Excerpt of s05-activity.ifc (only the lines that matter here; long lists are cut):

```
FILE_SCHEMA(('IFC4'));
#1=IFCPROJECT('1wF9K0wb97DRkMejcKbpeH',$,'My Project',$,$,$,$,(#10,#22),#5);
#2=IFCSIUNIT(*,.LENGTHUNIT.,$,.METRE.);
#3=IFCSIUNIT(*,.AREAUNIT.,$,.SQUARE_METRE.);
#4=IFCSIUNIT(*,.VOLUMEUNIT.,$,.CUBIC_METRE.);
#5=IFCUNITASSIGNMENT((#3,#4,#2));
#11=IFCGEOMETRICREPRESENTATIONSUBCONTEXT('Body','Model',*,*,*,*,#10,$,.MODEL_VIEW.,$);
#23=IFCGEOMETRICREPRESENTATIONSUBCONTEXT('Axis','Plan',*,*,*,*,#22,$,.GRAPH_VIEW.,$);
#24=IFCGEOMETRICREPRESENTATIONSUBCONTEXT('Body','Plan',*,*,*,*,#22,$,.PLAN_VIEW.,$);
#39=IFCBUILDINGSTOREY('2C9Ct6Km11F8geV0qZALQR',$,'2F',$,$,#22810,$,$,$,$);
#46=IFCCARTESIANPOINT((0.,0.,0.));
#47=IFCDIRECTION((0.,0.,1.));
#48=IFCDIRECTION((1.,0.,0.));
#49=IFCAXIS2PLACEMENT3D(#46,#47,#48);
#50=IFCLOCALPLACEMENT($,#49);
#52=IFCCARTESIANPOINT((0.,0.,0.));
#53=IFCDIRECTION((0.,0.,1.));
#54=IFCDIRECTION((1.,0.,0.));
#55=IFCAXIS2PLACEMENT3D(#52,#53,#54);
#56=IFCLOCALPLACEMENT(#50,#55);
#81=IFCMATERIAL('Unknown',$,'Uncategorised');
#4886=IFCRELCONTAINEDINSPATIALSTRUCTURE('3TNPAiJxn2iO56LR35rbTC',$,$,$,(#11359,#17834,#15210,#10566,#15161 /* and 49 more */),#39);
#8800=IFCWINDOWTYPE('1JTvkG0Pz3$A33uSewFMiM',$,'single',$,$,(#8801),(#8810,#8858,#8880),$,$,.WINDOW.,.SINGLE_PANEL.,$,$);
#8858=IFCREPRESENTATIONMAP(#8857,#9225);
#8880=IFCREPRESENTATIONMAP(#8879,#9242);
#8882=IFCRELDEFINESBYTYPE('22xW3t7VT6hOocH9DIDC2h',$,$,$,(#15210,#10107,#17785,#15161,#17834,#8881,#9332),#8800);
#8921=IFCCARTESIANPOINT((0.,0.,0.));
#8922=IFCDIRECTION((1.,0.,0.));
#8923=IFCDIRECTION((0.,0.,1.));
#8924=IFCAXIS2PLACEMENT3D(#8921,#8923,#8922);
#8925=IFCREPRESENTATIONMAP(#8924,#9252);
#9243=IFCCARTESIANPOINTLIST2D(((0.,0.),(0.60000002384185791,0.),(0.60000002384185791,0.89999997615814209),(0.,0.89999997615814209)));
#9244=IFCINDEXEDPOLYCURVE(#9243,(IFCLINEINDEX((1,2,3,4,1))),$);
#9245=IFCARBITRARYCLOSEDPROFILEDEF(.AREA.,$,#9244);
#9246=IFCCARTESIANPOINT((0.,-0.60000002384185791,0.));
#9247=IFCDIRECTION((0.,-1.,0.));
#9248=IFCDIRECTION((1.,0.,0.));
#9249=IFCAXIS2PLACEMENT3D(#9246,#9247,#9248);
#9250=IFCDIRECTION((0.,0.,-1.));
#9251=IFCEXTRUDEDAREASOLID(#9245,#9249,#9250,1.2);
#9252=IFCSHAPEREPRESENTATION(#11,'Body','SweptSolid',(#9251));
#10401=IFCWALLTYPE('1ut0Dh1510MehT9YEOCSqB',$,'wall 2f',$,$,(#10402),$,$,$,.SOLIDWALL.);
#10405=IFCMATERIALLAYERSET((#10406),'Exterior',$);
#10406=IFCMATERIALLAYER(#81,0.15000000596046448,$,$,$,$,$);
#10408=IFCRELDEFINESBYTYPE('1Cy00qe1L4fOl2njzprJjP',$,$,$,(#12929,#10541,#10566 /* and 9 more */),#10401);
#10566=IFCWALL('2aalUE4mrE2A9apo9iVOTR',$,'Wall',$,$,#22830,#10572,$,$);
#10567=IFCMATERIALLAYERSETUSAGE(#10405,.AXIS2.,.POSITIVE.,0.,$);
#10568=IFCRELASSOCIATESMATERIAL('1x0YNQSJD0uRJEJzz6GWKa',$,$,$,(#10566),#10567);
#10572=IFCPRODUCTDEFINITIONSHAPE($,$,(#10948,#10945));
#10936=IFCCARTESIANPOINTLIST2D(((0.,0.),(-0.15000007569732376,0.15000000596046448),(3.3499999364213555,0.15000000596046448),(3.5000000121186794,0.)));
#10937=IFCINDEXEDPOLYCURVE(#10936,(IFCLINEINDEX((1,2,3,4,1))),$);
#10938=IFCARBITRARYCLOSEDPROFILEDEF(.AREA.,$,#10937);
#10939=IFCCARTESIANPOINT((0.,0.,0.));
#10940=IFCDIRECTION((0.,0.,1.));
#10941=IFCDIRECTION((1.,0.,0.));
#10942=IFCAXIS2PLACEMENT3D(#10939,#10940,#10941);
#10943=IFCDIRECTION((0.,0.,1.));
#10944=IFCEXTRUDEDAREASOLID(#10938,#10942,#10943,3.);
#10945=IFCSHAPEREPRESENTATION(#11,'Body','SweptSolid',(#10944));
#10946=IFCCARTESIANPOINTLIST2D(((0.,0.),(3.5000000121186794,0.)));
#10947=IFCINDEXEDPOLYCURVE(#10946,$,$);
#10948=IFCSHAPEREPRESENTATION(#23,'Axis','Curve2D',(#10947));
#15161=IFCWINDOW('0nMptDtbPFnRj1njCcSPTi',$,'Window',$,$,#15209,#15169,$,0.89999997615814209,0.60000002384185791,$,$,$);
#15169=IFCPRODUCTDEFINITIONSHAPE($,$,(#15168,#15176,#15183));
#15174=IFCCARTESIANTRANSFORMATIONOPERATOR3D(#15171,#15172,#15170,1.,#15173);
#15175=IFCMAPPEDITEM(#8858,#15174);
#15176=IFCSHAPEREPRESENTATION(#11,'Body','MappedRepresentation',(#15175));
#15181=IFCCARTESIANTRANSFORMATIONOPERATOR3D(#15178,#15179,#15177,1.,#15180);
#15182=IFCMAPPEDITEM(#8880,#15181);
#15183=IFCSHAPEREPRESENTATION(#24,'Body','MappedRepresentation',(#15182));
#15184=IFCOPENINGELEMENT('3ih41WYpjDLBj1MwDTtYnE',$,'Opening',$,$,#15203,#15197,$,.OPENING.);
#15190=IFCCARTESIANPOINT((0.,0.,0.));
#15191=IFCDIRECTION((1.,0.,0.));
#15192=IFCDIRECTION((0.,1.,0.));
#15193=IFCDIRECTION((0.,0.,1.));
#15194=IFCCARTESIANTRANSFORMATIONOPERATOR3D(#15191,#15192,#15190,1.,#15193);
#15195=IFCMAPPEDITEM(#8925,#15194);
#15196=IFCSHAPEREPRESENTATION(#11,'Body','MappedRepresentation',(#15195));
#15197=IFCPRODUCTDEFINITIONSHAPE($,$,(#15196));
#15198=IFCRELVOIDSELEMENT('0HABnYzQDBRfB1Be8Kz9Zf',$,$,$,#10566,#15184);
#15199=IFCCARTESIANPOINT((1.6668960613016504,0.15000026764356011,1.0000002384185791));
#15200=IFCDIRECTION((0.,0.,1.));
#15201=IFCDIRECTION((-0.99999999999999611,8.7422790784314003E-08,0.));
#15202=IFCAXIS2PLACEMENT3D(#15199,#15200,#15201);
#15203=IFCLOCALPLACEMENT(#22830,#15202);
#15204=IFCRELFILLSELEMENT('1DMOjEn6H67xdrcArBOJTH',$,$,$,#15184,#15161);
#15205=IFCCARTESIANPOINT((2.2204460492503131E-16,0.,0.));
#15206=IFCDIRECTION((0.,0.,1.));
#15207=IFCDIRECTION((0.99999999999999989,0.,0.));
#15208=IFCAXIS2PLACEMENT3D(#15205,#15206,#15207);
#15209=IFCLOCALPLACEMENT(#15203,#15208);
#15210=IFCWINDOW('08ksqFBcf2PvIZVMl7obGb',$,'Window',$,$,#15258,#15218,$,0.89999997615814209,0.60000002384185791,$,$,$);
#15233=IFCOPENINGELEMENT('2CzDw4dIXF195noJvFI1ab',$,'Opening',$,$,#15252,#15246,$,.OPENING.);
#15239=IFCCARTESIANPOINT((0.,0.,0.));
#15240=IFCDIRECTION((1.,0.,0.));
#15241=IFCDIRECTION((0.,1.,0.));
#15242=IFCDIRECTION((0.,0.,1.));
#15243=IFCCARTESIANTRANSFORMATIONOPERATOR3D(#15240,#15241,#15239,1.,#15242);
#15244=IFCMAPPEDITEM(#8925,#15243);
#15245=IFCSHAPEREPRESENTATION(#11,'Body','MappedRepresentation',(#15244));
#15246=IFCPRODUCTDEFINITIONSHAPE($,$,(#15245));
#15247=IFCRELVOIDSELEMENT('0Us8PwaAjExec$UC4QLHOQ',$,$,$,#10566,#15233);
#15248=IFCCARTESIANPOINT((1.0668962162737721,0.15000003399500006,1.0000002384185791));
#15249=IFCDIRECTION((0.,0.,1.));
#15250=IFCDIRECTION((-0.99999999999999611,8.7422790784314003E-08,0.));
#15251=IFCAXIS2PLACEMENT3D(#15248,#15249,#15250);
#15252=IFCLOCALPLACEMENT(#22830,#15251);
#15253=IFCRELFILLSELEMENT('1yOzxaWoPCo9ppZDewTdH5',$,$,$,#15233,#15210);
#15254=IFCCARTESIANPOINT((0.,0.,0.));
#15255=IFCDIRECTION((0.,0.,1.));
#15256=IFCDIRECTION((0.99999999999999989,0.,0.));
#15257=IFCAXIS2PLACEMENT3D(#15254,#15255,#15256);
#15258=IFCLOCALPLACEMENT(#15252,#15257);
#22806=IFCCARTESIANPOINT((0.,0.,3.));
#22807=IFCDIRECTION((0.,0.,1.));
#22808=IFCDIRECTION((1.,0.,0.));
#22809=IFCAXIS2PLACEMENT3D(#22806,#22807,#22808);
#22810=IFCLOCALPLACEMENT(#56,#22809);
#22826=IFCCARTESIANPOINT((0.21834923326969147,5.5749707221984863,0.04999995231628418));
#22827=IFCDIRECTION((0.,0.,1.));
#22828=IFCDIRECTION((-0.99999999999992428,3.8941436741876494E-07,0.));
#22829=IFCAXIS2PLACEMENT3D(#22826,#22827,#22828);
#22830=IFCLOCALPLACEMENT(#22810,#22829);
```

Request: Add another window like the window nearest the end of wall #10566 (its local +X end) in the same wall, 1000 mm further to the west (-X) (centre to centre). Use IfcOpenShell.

```python
import ifcopenshell
import ifcopenshell.api.feature
import ifcopenshell.api.geometry
import ifcopenshell.api.root
import ifcopenshell.geom
import ifcopenshell.util.element
import ifcopenshell.util.placement
import ifcopenshell.util.shape
import ifcopenshell.util.unit

model = ifcopenshell.open("s05-activity.ifc")
unit_scale = ifcopenshell.util.unit.calculate_unit_scale(model)
settings = ifcopenshell.geom.settings()


def volume(element):
    """Net volume in cubic metres, openings subtracted."""
    shape = ifcopenshell.geom.create_shape(settings, element)
    return ifcopenshell.util.shape.get_volume(shape.geometry)


window = model.by_guid("0nMptDtbPFnRj1njCcSPTi")
opening = window.FillsVoids[0].RelatingOpeningElement
wall = opening.VoidsElements[0].RelatingBuildingElement
before = volume(wall)
shift = ifcopenshell.util.placement.get_local_placement(wall.ObjectPlacement)[:3, 0] * 1 / unit_scale

# copy_class copies the void relationship, type, container and properties, but no geometry.
new_opening = ifcopenshell.api.root.copy_class(model, product=opening)
new_opening.Representation = ifcopenshell.util.element.copy_deep(
    model, opening.Representation, exclude=["IfcGeometricRepresentationContext", "IfcRepresentationMap"]
)
new_window = ifcopenshell.api.root.copy_class(model, product=window)
new_window.Representation = ifcopenshell.util.element.copy_deep(
    model, window.Representation, exclude=["IfcGeometricRepresentationContext", "IfcRepresentationMap"]
)
ifcopenshell.api.feature.add_filling(model, opening=new_opening, element=new_window)

for old, new in ((opening, new_opening), (window, new_window)):
    matrix = ifcopenshell.util.placement.get_local_placement(old.ObjectPlacement)
    matrix[:3, 3] += shift
    ifcopenshell.api.geometry.edit_object_placement(model, product=new, matrix=matrix, is_si=False)

after = volume(wall)

print(f"wall volume {before:.3f} -> {after:.3f} m3")

model.write("s05-activity-out.ifc")
```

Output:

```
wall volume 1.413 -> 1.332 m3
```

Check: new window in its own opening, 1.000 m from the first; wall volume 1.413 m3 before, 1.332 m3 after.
